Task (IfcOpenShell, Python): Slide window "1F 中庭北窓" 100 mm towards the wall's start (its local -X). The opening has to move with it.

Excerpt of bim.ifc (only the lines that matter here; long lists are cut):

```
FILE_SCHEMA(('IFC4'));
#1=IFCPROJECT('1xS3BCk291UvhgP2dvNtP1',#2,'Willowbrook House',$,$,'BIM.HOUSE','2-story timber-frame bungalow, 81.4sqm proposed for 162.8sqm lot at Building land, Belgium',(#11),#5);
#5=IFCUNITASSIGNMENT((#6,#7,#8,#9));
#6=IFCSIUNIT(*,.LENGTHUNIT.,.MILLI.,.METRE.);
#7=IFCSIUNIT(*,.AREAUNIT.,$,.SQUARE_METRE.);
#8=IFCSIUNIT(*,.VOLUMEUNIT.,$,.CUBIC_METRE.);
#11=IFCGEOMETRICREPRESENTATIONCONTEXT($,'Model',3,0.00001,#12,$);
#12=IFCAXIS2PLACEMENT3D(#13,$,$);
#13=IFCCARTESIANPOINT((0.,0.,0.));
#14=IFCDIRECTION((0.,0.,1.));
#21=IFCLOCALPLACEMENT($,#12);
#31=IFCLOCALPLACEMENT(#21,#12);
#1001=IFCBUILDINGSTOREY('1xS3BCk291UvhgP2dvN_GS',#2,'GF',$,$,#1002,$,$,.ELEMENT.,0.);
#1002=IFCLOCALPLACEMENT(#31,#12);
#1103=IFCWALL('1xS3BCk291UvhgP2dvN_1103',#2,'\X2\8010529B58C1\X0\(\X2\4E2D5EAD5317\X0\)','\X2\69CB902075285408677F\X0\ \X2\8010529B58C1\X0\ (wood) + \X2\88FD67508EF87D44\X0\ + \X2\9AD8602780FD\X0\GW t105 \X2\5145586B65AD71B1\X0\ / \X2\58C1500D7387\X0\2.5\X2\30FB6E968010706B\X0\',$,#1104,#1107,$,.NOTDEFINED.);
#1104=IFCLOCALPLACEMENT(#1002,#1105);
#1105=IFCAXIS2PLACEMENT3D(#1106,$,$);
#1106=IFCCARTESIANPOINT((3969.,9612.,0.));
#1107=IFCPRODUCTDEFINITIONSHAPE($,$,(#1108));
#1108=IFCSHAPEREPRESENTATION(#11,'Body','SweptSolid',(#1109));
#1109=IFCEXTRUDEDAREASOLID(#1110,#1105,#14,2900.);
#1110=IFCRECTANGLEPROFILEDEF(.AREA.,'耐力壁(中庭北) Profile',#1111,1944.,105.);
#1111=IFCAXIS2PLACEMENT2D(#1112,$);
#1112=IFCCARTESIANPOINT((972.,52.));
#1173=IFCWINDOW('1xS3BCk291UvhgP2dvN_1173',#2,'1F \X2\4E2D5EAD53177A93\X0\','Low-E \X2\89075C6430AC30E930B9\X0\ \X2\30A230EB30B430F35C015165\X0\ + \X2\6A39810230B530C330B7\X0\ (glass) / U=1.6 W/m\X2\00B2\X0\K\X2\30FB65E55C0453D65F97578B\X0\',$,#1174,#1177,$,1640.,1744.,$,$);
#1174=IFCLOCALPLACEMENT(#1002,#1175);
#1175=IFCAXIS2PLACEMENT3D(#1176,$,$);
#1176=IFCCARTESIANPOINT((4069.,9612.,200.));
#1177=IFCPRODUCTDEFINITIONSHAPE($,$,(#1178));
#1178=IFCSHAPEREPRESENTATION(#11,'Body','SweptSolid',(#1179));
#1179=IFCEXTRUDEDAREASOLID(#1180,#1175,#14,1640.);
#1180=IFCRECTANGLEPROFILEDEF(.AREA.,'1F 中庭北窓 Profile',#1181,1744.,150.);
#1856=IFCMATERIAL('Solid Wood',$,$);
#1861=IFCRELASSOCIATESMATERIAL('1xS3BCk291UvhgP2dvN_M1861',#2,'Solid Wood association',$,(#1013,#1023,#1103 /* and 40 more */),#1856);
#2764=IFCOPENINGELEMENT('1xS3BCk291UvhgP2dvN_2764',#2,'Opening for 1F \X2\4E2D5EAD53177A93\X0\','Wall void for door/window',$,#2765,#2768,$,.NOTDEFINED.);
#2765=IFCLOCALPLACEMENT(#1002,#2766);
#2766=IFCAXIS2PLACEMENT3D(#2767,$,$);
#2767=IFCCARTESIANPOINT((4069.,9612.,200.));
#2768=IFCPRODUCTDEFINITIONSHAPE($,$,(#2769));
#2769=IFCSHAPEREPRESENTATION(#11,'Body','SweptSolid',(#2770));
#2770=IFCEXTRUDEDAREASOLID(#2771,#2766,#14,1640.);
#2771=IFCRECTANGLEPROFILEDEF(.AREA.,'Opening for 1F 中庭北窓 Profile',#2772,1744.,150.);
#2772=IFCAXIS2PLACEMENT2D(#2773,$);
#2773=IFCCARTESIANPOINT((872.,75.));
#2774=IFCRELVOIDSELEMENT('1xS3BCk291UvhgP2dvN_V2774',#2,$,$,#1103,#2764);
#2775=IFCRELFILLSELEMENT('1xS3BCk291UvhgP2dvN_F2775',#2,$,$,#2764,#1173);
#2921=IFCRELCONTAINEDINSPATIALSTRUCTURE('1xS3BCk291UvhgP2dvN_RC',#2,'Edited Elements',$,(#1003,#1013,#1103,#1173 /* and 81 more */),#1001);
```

```python
import ifcopenshell
import ifcopenshell.api.geometry
import ifcopenshell.util.placement

model = ifcopenshell.open("bim.ifc")

window = model.by_guid("1xS3BCk291UvhgP2dvN_1173")
opening = window.FillsVoids[0].RelatingOpeningElement
wall = opening.VoidsElements[0].RelatingBuildingElement

wall_matrix = ifcopenshell.util.placement.get_local_placement(wall.ObjectPlacement)
shift = wall_matrix[:3, 0] * -100.0
before = ifcopenshell.util.placement.get_local_placement(window.ObjectPlacement)[:3, 3].copy()

# The window is not placed relative to its opening, so move both.
for product in (opening, window):
    matrix = ifcopenshell.util.placement.get_local_placement(product.ObjectPlacement)
    matrix[:3, 3] += shift
    ifcopenshell.api.geometry.edit_object_placement(model, product=product, matrix=matrix, is_si=False)

after = ifcopenshell.util.placement.get_local_placement(window.ObjectPlacement)[:3, 3]
print("window moved by", (after - before).round(3) + 0.0)

model.write("bim_rev.ifc")
```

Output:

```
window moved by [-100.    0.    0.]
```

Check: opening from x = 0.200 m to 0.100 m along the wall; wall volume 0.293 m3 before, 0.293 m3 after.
